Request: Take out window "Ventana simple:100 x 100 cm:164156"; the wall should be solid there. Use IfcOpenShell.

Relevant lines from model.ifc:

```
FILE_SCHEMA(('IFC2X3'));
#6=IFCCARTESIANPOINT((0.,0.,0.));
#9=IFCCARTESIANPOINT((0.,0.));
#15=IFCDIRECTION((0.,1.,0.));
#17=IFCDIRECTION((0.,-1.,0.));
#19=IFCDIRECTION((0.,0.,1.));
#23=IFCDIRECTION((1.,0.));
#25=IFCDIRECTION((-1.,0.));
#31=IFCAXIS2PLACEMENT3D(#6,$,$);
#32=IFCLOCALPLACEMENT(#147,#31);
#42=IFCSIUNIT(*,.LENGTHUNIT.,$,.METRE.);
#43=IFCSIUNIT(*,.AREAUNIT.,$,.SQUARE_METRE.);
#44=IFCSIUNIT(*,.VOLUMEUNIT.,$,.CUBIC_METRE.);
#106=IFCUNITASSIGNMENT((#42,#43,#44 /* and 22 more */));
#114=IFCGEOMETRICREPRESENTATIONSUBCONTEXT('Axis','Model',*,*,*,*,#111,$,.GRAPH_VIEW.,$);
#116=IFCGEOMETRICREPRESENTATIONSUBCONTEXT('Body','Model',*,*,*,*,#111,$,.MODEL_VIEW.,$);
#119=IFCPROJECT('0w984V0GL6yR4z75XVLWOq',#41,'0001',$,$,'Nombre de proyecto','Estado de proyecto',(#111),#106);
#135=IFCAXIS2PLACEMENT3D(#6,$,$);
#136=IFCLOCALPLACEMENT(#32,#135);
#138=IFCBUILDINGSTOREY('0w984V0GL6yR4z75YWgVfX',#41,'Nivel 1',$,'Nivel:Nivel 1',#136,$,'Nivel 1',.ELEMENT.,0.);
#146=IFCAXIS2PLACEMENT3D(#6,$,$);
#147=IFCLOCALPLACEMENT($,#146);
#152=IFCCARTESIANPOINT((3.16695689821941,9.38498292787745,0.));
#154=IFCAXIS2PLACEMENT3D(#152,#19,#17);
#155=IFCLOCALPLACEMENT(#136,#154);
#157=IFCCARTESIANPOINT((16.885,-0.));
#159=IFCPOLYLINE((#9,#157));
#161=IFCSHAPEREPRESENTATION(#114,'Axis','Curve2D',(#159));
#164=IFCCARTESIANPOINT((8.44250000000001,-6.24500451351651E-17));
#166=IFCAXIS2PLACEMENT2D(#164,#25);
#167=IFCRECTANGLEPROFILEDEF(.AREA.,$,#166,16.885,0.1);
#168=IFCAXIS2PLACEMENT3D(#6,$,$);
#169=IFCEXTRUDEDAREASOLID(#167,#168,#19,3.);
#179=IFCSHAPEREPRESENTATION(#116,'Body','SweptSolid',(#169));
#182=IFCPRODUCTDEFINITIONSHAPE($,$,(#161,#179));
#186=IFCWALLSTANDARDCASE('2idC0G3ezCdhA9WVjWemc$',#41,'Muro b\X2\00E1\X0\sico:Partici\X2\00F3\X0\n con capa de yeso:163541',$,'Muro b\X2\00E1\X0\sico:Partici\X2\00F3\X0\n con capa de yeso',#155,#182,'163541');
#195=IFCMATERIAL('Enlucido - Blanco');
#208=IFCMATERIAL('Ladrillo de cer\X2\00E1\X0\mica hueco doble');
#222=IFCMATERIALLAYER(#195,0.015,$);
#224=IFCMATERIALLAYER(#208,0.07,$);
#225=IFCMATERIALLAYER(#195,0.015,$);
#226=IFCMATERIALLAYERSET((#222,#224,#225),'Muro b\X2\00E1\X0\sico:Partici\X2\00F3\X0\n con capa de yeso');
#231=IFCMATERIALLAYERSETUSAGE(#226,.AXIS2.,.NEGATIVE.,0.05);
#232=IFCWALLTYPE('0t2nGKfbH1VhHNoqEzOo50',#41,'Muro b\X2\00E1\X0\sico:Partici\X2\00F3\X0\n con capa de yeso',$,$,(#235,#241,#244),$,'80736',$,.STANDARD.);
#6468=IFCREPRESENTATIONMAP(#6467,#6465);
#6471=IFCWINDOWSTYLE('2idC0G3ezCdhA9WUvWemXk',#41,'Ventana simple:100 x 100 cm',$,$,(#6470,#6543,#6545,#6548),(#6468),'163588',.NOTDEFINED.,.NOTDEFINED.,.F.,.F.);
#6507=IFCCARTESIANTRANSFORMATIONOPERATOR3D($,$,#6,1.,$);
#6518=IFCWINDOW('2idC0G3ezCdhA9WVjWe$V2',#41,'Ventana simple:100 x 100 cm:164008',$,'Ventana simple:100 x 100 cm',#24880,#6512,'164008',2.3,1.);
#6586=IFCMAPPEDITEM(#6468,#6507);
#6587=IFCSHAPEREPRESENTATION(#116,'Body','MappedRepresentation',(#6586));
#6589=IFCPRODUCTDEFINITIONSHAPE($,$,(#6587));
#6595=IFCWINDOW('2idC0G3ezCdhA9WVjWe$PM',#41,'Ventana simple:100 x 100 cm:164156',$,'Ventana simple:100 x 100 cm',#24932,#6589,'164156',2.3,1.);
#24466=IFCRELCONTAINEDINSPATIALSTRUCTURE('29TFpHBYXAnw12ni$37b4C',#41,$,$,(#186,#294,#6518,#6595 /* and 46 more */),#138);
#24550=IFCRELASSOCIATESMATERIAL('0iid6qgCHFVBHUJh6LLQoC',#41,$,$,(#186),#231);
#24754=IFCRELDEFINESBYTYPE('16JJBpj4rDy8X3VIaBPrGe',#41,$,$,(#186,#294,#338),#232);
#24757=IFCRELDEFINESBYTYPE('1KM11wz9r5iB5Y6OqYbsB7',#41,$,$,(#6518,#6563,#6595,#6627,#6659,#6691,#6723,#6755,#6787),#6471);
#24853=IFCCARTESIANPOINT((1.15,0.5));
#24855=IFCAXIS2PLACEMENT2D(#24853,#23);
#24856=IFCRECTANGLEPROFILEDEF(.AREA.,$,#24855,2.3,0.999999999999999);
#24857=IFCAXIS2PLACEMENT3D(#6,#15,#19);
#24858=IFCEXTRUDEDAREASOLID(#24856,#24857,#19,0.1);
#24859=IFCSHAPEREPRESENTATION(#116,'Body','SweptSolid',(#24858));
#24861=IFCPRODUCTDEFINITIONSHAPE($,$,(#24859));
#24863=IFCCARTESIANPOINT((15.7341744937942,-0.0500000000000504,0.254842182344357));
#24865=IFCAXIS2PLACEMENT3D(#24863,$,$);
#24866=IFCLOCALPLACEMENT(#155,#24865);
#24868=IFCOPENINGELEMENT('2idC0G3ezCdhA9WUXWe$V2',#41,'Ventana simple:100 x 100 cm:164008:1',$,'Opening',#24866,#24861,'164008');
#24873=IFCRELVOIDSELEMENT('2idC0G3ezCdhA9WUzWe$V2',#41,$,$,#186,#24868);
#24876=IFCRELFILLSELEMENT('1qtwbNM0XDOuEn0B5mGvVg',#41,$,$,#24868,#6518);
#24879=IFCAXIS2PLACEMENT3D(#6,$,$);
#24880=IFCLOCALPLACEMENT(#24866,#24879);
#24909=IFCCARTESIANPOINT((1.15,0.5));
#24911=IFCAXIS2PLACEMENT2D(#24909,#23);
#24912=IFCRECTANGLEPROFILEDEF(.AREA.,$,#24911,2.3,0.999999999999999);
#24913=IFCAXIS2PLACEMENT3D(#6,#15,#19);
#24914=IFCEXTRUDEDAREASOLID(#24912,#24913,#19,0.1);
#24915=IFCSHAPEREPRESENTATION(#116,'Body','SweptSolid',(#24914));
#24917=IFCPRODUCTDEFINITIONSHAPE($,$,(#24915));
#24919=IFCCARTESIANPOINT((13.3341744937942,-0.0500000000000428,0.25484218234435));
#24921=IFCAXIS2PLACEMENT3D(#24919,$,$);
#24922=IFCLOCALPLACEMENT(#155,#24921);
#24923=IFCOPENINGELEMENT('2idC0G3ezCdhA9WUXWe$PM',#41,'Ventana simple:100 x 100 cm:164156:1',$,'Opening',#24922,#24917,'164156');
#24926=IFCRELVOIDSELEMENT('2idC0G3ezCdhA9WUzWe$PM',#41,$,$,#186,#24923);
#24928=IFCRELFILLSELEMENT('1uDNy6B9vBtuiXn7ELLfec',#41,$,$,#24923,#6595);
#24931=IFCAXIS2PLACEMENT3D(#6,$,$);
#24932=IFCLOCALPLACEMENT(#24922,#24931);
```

```python
import ifcopenshell
import ifcopenshell.api.feature
import ifcopenshell.api.root
import ifcopenshell.geom
import ifcopenshell.util.shape

model = ifcopenshell.open("model.ifc")
settings = ifcopenshell.geom.settings()


def volume(element):
    """Net volume in cubic metres, openings subtracted."""
    shape = ifcopenshell.geom.create_shape(settings, element)
    return ifcopenshell.util.shape.get_volume(shape.geometry)


window = model.by_guid("2idC0G3ezCdhA9WVjWe$PM")
opening = window.FillsVoids[0].RelatingOpeningElement
wall = opening.VoidsElements[0].RelatingBuildingElement
before = volume(wall)

ifcopenshell.api.root.remove_product(model, product=window)
ifcopenshell.api.feature.remove_feature(model, feature=opening)

after = volume(wall)

print(f"wall volume {before:.3f} -> {after:.3f} m3")

model.write("model-out.ifc")
```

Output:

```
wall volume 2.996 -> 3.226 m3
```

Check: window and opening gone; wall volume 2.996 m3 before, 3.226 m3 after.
